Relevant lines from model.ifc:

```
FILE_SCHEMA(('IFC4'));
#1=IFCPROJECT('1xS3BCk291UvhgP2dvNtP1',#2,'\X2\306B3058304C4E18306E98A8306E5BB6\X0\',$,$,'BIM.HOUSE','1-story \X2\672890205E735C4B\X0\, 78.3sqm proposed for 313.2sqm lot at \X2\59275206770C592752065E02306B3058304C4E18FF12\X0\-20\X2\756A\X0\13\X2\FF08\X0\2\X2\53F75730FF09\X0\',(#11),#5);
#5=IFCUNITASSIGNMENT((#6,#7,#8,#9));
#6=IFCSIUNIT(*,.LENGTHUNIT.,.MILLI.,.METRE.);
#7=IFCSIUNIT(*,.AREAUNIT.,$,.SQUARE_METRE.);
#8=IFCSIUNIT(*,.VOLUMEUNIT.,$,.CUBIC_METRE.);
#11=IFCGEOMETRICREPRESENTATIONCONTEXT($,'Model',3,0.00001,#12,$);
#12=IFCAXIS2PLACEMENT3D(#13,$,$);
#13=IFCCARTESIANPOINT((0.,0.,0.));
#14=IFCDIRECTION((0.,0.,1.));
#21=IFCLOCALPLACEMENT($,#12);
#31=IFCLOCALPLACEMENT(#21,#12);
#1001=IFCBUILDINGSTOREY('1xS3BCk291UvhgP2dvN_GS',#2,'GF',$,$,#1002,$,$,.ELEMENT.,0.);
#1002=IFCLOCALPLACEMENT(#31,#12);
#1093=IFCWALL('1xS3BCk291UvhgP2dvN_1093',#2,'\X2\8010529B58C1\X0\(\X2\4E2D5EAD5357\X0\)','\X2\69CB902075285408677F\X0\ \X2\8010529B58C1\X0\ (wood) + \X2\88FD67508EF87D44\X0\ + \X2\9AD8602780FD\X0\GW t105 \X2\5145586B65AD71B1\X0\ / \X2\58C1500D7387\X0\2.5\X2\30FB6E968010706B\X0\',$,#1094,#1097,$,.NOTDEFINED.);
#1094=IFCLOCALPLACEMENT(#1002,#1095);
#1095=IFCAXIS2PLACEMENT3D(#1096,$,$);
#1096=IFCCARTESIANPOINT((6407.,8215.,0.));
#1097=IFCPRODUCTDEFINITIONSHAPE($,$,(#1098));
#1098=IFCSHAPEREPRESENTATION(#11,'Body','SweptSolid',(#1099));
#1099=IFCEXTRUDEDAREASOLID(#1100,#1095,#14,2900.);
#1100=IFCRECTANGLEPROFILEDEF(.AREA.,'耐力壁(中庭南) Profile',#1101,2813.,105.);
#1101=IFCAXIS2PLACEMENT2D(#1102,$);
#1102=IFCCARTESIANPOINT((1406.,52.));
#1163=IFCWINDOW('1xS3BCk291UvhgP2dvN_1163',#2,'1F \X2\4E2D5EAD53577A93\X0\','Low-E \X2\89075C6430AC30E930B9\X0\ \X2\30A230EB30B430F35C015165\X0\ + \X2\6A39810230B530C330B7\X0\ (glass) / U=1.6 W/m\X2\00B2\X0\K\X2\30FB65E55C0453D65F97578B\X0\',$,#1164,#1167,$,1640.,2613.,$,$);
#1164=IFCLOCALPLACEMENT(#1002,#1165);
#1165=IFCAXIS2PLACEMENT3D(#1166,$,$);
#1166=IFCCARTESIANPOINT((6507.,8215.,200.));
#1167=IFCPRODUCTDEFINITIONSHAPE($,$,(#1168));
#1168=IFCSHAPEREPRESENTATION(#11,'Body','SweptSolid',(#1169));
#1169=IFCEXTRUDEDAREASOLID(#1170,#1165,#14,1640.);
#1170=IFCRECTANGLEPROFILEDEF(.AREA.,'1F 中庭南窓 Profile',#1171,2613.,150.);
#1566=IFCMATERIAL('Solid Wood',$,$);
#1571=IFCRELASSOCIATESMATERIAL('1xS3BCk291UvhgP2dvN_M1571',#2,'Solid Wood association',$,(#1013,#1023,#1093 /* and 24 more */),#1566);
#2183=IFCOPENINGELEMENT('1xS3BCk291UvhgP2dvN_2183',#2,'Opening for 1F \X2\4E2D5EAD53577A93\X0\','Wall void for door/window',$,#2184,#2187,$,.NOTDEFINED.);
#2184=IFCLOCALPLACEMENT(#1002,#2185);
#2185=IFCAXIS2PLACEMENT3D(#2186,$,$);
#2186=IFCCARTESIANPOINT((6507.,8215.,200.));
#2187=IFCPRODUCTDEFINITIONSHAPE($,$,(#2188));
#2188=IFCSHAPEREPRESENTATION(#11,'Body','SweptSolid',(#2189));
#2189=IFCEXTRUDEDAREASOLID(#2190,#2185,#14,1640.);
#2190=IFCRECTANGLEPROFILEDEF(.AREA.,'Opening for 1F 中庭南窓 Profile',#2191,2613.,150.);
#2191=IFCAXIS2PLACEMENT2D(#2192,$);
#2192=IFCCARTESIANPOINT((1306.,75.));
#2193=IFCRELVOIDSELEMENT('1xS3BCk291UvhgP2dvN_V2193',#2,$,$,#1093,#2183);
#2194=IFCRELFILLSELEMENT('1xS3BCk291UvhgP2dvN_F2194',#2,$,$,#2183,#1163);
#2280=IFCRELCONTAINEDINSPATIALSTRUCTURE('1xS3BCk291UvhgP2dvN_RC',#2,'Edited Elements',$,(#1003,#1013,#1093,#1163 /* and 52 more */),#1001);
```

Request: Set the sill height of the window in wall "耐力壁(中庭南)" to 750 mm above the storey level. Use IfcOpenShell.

```python
import numpy as np
import ifcopenshell
import ifcopenshell.api.geometry
import ifcopenshell.geom
import ifcopenshell.util.element
import ifcopenshell.util.placement
import ifcopenshell.util.shape
import ifcopenshell.util.unit

model = ifcopenshell.open("model.ifc")
unit_scale = ifcopenshell.util.unit.calculate_unit_scale(model)

window = model.by_id(1163)
opening = window.FillsVoids[0].RelatingOpeningElement
storey = ifcopenshell.util.element.get_container(window, ifc_class="IfcBuildingStorey")
level = ifcopenshell.util.placement.get_local_placement(storey.ObjectPlacement)[2, 3]

# The opening's origin need not be at the sill, so measure its lowest point.
shape = ifcopenshell.geom.create_shape(ifcopenshell.geom.settings(), opening)
bottom = ifcopenshell.util.shape.get_shape_bottom_elevation(shape, shape.geometry) / unit_scale
dz = level + 750.0 - bottom

shift = np.array([0.0, 0.0, dz])
# The window is not placed relative to its opening, so move both.
for product in (opening, window):
    matrix = ifcopenshell.util.placement.get_local_placement(product.ObjectPlacement)
    matrix[:3, 3] += shift
    ifcopenshell.api.geometry.edit_object_placement(model, product=product, matrix=matrix, is_si=False)

print(f"moved by {dz * unit_scale:+.3f} m")

model.write("model_updated.ifc")
```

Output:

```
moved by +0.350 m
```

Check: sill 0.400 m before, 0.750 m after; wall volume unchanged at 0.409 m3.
